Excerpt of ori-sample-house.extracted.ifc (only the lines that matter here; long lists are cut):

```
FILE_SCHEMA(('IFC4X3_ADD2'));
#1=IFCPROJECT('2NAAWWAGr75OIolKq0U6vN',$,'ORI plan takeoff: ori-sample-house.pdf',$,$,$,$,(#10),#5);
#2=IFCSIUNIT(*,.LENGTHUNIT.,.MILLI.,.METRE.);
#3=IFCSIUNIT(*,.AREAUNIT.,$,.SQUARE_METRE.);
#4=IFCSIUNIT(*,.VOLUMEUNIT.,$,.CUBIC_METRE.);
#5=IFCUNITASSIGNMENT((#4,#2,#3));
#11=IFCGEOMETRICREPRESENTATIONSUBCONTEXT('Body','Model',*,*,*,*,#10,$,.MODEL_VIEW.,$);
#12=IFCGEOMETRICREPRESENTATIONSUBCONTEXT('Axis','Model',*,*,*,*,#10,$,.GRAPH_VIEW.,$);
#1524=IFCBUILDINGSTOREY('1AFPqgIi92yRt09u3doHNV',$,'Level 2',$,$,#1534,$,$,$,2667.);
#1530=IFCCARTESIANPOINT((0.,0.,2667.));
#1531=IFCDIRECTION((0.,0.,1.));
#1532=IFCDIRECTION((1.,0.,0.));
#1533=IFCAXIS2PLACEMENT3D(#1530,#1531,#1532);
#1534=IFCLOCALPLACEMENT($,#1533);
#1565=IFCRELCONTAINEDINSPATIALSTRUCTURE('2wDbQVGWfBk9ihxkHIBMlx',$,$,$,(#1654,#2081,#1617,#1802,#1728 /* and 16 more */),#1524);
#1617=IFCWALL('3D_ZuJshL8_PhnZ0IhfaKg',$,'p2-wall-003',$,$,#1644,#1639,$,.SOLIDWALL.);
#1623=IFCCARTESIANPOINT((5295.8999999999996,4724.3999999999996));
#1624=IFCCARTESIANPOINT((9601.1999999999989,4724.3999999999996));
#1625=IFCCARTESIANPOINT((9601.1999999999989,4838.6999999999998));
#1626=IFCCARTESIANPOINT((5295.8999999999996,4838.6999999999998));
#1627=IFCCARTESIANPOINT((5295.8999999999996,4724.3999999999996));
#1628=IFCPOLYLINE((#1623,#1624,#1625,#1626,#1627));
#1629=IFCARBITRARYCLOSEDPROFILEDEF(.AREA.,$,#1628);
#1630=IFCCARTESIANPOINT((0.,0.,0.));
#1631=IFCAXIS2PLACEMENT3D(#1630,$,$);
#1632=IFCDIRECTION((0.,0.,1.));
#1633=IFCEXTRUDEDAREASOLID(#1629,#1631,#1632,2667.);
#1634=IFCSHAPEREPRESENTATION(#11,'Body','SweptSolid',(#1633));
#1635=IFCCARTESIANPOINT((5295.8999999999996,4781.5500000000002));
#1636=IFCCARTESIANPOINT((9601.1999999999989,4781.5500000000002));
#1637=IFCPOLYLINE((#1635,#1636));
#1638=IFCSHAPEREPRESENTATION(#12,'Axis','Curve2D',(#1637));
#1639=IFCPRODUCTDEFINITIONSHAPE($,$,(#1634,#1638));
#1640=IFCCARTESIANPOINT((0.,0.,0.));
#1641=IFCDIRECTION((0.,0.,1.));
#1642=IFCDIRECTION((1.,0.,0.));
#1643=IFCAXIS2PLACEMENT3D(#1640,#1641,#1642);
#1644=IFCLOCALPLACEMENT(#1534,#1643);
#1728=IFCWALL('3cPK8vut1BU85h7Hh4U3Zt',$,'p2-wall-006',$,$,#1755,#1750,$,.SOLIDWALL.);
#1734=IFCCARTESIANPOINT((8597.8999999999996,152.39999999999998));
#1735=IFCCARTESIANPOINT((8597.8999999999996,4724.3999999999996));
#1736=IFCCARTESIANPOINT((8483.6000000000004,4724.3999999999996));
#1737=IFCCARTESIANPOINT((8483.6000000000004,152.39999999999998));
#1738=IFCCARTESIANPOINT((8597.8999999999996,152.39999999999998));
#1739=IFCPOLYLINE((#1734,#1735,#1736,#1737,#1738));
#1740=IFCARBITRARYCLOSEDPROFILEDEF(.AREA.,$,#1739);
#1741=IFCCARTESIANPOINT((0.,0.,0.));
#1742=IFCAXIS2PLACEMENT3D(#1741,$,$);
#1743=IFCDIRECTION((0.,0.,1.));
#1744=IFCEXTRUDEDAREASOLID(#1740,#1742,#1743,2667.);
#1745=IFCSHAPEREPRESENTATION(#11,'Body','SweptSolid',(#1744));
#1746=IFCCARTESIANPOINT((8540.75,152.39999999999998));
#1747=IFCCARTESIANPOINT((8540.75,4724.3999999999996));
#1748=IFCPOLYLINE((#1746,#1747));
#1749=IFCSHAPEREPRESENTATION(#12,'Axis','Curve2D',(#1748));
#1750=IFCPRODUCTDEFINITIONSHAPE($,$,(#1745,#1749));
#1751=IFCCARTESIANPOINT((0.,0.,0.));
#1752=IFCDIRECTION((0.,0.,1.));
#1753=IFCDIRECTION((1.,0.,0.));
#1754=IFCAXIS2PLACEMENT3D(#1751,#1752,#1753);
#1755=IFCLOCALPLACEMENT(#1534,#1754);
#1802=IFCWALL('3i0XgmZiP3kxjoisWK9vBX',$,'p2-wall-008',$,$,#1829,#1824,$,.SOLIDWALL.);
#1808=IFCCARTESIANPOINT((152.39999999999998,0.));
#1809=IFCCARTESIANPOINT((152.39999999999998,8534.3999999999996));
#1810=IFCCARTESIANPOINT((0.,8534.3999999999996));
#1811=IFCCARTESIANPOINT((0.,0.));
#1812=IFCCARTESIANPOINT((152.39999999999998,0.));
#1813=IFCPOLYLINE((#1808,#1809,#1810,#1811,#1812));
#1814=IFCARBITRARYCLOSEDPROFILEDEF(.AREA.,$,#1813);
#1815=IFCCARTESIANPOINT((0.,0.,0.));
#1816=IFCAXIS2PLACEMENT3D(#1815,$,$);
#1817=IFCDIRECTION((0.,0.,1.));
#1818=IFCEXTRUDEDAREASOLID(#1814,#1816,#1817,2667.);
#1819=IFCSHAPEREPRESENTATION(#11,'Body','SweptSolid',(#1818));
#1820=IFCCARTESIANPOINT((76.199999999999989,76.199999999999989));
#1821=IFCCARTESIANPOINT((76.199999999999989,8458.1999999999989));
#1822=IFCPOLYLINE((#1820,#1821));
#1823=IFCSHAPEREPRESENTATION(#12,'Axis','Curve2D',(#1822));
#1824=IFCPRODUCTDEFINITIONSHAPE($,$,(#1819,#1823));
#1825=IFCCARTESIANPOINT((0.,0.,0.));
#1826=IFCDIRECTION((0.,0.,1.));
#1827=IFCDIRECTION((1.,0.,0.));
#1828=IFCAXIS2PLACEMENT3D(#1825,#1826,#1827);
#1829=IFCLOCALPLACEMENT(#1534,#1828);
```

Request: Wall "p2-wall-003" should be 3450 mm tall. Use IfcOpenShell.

```python
import ifcopenshell
import ifcopenshell.geom
import ifcopenshell.util.representation
import ifcopenshell.util.shape
import ifcopenshell.util.unit

model = ifcopenshell.open("ori-sample-house.extracted.ifc")
unit_scale = ifcopenshell.util.unit.calculate_unit_scale(model)
settings = ifcopenshell.geom.settings()


def volume(element):
    """Net volume in cubic metres, openings subtracted."""
    shape = ifcopenshell.geom.create_shape(settings, element)
    return ifcopenshell.util.shape.get_volume(shape.geometry)


wall = model.by_id(1617)
before = volume(wall)

body = ifcopenshell.util.representation.get_representation(wall, "Model", "Body")
solid = body.Items[0]
old_height = solid.Depth
solid.Depth = 3.45 / unit_scale
after = volume(wall)

print(f"height {old_height:g} -> {solid.Depth:g}, volume {before:.3f} -> {after:.3f} m3")

model.write("ori-sample-house.extracted_updated.ifc")
```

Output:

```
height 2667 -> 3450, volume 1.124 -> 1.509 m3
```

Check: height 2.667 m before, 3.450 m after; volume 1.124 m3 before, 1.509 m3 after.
